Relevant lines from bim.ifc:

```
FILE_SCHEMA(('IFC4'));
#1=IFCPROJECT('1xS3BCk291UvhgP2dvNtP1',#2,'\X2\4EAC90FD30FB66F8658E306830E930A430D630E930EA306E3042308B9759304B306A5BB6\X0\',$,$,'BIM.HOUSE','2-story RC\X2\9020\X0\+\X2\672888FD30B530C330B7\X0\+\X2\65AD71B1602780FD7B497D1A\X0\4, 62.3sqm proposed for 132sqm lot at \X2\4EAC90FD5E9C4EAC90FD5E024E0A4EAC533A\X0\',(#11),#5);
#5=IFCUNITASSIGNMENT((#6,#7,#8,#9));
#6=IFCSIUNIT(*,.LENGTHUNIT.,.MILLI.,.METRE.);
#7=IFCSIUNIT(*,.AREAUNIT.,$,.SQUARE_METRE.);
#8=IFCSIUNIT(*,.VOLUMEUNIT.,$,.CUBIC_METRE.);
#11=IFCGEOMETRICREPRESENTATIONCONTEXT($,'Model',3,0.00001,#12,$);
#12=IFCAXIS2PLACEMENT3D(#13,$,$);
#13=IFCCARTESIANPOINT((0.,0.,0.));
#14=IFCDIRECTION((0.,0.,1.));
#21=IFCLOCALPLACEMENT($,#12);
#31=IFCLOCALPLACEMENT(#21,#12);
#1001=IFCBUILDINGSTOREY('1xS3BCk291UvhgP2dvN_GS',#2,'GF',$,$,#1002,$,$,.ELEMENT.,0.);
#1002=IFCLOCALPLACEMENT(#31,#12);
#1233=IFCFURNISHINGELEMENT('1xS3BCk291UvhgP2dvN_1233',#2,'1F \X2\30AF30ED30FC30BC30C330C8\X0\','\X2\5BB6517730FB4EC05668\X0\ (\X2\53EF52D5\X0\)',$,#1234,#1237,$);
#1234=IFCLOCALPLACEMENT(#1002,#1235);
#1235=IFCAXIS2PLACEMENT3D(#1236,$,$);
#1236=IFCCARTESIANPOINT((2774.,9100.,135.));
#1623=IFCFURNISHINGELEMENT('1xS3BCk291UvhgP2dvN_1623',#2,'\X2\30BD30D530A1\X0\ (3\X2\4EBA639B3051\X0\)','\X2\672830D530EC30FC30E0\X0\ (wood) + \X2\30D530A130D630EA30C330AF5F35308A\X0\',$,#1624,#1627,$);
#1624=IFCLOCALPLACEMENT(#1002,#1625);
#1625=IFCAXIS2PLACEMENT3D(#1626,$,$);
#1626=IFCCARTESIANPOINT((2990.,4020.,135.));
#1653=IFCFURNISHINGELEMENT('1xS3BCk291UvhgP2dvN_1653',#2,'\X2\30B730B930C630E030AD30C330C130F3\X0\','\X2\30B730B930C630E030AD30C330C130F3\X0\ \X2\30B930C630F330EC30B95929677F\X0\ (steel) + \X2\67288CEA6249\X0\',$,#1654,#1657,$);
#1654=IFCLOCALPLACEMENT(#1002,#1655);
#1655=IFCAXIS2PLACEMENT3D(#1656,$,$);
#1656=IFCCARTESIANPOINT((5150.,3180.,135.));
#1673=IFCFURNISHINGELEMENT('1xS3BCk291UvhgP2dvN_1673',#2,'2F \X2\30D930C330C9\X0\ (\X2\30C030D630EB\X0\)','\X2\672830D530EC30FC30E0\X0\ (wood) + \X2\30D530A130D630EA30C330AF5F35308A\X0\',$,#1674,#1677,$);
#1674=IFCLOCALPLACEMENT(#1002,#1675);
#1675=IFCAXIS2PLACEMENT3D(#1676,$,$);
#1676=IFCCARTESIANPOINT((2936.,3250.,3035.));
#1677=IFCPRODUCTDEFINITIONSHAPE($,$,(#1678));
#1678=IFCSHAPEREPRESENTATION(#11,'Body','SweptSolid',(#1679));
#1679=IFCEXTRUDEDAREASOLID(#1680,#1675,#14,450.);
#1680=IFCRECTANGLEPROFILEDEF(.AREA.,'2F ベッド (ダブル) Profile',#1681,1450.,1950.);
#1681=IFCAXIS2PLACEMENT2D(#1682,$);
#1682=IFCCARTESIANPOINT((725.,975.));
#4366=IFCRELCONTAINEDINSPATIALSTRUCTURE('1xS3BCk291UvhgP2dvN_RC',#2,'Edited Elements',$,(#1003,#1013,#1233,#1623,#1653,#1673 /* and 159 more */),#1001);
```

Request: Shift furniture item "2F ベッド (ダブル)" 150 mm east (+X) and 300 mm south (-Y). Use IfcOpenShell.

```python
import ifcopenshell
import ifcopenshell.api.geometry
import ifcopenshell.util.placement

model = ifcopenshell.open("bim.ifc")

item = model.by_id(1673)
matrix = ifcopenshell.util.placement.get_local_placement(item.ObjectPlacement)
matrix[0, 3] += 150.0
matrix[1, 3] -= 300.0
ifcopenshell.api.geometry.edit_object_placement(model, product=item, matrix=matrix, is_si=False)

print(ifcopenshell.util.placement.get_local_placement(item.ObjectPlacement).round(3) + 0.0)

model.write("bim-out.ifc")
```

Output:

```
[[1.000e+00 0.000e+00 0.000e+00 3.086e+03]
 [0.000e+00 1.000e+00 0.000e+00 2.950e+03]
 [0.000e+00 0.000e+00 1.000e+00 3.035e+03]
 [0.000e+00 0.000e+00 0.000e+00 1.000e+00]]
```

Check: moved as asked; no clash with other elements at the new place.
